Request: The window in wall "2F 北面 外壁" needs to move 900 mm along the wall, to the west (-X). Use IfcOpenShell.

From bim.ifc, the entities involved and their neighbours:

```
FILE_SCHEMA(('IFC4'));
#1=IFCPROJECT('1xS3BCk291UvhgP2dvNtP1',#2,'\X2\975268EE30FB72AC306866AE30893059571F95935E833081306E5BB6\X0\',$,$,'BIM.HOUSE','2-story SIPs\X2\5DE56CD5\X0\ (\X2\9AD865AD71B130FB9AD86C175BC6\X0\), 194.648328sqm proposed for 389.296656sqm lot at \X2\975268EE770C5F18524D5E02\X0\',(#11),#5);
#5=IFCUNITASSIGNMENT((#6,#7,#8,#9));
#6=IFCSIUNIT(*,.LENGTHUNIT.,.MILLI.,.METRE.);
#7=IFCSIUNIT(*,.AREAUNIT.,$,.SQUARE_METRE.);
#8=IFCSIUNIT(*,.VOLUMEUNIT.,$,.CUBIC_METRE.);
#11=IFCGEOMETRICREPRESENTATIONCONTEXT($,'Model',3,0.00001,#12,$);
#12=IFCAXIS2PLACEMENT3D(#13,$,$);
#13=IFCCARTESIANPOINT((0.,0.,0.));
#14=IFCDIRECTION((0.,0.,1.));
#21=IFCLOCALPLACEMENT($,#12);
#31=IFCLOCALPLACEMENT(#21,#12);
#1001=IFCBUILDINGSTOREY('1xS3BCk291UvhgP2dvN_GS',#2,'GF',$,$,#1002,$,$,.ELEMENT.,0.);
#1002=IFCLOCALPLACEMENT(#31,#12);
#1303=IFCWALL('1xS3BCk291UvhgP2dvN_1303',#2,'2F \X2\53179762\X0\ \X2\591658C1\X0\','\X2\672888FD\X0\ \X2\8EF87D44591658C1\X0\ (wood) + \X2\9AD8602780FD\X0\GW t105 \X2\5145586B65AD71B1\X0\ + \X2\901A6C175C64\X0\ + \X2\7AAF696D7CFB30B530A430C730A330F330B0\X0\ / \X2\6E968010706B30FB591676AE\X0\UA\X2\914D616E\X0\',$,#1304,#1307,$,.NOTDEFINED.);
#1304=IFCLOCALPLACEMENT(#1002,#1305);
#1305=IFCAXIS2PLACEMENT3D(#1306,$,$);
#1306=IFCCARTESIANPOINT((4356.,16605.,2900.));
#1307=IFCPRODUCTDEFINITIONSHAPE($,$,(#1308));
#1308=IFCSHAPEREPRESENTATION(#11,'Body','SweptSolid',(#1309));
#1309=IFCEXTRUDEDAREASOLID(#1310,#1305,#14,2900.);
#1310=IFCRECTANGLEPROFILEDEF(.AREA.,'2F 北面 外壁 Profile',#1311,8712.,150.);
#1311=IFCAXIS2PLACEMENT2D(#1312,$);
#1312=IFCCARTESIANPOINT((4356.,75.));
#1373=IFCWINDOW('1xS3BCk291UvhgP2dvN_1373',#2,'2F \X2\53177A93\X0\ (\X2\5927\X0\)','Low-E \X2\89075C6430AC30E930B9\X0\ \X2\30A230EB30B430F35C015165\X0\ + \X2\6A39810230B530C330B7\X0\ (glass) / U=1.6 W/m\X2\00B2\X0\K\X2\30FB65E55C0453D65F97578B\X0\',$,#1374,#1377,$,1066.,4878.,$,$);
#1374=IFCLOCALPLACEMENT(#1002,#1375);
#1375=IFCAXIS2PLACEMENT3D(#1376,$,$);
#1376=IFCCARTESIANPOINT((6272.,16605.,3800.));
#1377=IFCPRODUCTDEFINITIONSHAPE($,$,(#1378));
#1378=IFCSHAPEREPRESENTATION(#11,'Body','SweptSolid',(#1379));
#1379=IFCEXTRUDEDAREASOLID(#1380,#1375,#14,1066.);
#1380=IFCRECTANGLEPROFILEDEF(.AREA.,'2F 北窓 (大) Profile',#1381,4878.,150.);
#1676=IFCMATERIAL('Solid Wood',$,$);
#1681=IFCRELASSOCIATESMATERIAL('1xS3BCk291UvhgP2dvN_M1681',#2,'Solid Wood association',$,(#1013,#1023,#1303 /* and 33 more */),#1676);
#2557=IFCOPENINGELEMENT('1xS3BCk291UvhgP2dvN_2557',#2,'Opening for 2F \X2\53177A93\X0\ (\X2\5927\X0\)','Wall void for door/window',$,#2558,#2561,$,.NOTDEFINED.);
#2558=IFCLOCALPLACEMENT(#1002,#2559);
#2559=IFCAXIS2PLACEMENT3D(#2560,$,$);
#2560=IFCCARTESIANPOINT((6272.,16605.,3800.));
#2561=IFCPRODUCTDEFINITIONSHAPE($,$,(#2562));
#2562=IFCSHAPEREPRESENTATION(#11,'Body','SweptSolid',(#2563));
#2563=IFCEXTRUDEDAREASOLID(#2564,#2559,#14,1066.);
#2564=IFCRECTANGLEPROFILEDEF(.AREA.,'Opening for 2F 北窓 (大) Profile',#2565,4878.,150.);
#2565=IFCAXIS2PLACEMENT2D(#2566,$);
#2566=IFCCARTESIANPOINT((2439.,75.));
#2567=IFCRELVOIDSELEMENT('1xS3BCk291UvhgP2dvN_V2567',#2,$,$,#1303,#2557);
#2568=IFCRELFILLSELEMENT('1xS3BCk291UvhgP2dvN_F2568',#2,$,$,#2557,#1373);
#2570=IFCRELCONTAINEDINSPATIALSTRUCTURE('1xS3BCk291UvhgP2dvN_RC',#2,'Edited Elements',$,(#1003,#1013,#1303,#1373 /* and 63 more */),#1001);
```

```python
import ifcopenshell
import ifcopenshell.api.geometry
import ifcopenshell.util.placement
import ifcopenshell.util.unit

model = ifcopenshell.open("bim.ifc")
unit_scale = ifcopenshell.util.unit.calculate_unit_scale(model)

window = model.by_guid("1xS3BCk291UvhgP2dvN_1373")
opening = window.FillsVoids[0].RelatingOpeningElement
wall = opening.VoidsElements[0].RelatingBuildingElement

wall_matrix = ifcopenshell.util.placement.get_local_placement(wall.ObjectPlacement)
shift = wall_matrix[:3, 0] * -0.9 / unit_scale
before = ifcopenshell.util.placement.get_local_placement(window.ObjectPlacement)[:3, 3].copy()

# The window is not placed relative to its opening, so move both.
for product in (opening, window):
    matrix = ifcopenshell.util.placement.get_local_placement(product.ObjectPlacement)
    matrix[:3, 3] += shift
    ifcopenshell.api.geometry.edit_object_placement(model, product=product, matrix=matrix, is_si=False)

after = ifcopenshell.util.placement.get_local_placement(window.ObjectPlacement)[:3, 3]
print("window moved by", (after - before).round(3) + 0.0)

model.write("bim_edited.ifc")
```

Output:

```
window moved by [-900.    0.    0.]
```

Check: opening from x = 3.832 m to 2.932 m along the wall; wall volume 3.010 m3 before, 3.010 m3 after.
